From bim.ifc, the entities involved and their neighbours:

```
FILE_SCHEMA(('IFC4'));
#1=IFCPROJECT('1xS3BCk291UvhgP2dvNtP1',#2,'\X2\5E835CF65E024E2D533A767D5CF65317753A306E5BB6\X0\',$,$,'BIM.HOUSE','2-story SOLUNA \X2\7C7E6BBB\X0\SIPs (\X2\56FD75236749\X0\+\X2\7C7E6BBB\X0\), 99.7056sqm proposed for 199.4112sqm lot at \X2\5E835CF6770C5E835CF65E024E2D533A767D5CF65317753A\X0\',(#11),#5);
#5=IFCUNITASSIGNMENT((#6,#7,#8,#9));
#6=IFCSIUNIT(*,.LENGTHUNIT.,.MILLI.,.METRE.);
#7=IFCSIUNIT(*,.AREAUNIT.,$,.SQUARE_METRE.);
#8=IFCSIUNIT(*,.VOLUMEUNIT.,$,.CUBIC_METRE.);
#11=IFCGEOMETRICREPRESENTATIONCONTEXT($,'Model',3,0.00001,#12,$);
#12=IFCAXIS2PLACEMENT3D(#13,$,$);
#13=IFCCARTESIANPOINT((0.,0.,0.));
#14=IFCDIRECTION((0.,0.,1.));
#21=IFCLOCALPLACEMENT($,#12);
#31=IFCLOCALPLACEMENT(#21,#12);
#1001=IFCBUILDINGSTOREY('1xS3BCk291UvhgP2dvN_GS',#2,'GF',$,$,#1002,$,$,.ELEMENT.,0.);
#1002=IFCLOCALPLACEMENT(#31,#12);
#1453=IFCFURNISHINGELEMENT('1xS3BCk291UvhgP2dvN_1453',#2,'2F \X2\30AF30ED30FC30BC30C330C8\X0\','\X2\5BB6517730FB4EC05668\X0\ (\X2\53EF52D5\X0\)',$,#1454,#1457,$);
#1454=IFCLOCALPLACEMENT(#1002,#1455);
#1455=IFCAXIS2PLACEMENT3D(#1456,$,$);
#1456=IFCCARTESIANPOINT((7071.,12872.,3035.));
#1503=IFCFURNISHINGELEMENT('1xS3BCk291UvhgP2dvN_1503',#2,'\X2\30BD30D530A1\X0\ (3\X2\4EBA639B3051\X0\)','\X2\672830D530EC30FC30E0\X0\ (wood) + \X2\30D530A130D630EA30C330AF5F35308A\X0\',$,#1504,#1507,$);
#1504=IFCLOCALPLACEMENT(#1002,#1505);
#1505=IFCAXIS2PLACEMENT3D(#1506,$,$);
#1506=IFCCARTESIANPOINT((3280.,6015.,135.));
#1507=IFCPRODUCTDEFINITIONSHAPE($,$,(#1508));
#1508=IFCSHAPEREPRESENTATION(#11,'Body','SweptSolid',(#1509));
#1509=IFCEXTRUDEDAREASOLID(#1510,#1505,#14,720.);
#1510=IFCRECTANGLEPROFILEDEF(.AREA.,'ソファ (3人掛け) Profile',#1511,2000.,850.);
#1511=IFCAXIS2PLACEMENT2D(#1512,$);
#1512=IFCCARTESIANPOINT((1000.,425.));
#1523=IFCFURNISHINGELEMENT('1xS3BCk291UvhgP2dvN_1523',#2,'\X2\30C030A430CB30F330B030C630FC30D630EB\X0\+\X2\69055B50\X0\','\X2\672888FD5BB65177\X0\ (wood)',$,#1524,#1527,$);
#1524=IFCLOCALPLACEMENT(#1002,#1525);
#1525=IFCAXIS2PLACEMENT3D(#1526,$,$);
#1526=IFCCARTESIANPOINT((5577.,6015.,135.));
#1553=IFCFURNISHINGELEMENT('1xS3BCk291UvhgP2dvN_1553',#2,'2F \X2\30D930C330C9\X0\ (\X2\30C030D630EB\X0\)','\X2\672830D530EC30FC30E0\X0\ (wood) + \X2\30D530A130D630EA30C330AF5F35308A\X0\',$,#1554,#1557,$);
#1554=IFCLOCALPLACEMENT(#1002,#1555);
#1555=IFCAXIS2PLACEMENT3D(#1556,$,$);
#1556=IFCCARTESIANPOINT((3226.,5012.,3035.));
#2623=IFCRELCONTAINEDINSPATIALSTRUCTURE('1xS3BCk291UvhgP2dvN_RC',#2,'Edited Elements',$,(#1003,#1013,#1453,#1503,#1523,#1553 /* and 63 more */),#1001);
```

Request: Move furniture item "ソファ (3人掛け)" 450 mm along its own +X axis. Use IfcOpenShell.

```python
import ifcopenshell
import ifcopenshell.api.geometry
import ifcopenshell.util.placement
import ifcopenshell.util.unit

model = ifcopenshell.open("bim.ifc")
unit_scale = ifcopenshell.util.unit.calculate_unit_scale(model)

item = model.by_guid("1xS3BCk291UvhgP2dvN_1503")
matrix = ifcopenshell.util.placement.get_local_placement(item.ObjectPlacement)
matrix[:3, 3] += matrix[:3, 0] * 0.45 / unit_scale
ifcopenshell.api.geometry.edit_object_placement(model, product=item, matrix=matrix, is_si=False)

print(ifcopenshell.util.placement.get_local_placement(item.ObjectPlacement).round(3) + 0.0)

model.write("bim_v2.ifc")
```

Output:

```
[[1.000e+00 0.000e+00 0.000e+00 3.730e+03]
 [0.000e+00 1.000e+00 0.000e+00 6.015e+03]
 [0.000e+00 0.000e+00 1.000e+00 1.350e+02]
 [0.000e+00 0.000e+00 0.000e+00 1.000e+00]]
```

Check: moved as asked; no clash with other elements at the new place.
